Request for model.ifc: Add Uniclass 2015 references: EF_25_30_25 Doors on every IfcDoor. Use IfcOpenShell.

First a look at what the model holds.

```python
import ifcopenshell

model = ifcopenshell.open("model.ifc")
print(model.schema)
print("classifications:", [c.Name for c in model.by_type("IfcClassification")])
for ifc_class in ("IfcDoor", "IfcRoof", "IfcStair", "IfcWall", "IfcWindow"):
    print(ifc_class, len(model.by_type(ifc_class)))
```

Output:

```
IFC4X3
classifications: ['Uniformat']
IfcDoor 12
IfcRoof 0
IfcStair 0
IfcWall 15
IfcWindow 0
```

```python
import ifcopenshell
import ifcopenshell.api.classification

model = ifcopenshell.open("model.ifc")

system = ifcopenshell.api.classification.add_classification(model, classification="Uniclass 2015")

codes = {
    "IfcDoor": ("EF_25_30_25", "Doors"),
}
for ifc_class, (code, name) in codes.items():
    products = model.by_type(ifc_class)
    ifcopenshell.api.classification.add_reference(
        model, products=products, classification=system, identification=code, name=name
    )
    print(code, len(products))

model.write("model_updated.ifc")
```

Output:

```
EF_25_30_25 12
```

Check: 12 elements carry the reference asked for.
